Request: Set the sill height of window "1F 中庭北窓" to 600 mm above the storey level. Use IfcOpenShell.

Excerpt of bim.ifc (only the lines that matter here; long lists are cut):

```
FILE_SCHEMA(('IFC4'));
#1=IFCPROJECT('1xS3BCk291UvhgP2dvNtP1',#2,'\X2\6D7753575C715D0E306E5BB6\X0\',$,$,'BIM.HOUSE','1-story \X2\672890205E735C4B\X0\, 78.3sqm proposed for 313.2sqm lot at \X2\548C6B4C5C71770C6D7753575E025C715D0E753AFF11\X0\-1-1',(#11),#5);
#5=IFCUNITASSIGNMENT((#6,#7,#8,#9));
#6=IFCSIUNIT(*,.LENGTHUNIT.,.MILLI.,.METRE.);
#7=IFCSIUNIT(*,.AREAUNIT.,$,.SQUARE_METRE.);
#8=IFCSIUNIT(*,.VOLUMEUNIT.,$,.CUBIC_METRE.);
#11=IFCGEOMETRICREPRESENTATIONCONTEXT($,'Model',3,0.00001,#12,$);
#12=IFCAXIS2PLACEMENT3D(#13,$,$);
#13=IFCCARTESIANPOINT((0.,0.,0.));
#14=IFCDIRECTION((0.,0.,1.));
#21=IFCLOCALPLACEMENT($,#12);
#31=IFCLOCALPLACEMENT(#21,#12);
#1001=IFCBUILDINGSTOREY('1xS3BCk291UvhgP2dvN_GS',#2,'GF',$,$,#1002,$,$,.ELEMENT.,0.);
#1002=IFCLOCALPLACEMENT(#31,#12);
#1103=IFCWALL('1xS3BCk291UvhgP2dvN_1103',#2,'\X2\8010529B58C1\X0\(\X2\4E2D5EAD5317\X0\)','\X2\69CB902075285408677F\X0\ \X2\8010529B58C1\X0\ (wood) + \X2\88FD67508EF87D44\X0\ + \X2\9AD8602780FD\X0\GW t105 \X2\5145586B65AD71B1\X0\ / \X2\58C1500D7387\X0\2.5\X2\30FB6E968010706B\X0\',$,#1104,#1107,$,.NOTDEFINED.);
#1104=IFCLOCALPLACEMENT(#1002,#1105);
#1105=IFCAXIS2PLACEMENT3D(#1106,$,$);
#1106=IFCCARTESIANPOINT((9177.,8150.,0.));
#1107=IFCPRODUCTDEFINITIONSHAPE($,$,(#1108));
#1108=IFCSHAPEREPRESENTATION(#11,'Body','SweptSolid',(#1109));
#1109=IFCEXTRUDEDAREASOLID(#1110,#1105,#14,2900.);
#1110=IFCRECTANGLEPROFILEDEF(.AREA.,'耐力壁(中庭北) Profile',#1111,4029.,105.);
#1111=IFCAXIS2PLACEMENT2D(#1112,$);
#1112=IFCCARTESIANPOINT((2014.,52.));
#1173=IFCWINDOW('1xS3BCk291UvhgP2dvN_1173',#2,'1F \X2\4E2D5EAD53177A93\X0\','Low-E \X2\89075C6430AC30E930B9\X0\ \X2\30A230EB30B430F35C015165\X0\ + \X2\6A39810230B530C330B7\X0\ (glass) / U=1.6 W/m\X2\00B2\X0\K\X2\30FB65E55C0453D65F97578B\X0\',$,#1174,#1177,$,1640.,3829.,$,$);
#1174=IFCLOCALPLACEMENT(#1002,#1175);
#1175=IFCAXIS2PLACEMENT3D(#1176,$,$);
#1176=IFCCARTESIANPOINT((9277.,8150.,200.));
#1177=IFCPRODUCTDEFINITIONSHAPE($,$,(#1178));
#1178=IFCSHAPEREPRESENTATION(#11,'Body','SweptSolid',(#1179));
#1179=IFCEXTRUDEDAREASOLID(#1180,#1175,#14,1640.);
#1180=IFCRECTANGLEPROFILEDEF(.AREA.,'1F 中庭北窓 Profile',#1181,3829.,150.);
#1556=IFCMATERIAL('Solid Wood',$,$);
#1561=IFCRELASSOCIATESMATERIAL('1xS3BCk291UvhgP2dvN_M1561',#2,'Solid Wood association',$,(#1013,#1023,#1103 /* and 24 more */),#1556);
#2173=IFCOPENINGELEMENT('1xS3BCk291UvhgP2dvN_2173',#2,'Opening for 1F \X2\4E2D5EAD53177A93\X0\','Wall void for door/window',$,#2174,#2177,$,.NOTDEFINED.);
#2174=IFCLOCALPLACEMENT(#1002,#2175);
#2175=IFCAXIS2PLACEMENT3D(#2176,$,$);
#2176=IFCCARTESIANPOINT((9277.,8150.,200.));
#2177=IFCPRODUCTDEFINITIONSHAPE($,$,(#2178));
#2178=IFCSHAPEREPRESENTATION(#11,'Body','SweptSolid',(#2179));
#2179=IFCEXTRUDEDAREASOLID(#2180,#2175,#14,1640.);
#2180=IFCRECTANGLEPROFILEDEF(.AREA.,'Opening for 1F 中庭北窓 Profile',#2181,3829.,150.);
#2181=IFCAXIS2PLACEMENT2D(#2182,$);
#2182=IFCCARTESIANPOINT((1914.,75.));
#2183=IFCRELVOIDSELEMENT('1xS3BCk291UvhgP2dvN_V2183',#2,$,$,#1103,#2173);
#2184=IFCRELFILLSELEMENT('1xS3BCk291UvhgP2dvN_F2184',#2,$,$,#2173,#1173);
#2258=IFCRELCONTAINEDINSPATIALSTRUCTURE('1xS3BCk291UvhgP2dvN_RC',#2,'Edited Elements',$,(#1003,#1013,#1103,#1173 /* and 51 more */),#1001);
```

```python
import numpy as np
import ifcopenshell
import ifcopenshell.api.geometry
import ifcopenshell.geom
import ifcopenshell.util.element
import ifcopenshell.util.placement
import ifcopenshell.util.shape
import ifcopenshell.util.unit

model = ifcopenshell.open("bim.ifc")
unit_scale = ifcopenshell.util.unit.calculate_unit_scale(model)

window = model.by_id(1173)
opening = window.FillsVoids[0].RelatingOpeningElement
storey = ifcopenshell.util.element.get_container(window, ifc_class="IfcBuildingStorey")
level = ifcopenshell.util.placement.get_local_placement(storey.ObjectPlacement)[2, 3]

# The opening's origin need not be at the sill, so measure its lowest point.
shape = ifcopenshell.geom.create_shape(ifcopenshell.geom.settings(), opening)
bottom = ifcopenshell.util.shape.get_shape_bottom_elevation(shape, shape.geometry) / unit_scale
dz = level + 0.6 / unit_scale - bottom

shift = np.array([0.0, 0.0, dz])
# The window is not placed relative to its opening, so move both.
for product in (opening, window):
    matrix = ifcopenshell.util.placement.get_local_placement(product.ObjectPlacement)
    matrix[:3, 3] += shift
    ifcopenshell.api.geometry.edit_object_placement(model, product=product, matrix=matrix, is_si=False)

print(f"moved by {dz * unit_scale:+.3f} m")

model.write("bim_edited.ifc")
```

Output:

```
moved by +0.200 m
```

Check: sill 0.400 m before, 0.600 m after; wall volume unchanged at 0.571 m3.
